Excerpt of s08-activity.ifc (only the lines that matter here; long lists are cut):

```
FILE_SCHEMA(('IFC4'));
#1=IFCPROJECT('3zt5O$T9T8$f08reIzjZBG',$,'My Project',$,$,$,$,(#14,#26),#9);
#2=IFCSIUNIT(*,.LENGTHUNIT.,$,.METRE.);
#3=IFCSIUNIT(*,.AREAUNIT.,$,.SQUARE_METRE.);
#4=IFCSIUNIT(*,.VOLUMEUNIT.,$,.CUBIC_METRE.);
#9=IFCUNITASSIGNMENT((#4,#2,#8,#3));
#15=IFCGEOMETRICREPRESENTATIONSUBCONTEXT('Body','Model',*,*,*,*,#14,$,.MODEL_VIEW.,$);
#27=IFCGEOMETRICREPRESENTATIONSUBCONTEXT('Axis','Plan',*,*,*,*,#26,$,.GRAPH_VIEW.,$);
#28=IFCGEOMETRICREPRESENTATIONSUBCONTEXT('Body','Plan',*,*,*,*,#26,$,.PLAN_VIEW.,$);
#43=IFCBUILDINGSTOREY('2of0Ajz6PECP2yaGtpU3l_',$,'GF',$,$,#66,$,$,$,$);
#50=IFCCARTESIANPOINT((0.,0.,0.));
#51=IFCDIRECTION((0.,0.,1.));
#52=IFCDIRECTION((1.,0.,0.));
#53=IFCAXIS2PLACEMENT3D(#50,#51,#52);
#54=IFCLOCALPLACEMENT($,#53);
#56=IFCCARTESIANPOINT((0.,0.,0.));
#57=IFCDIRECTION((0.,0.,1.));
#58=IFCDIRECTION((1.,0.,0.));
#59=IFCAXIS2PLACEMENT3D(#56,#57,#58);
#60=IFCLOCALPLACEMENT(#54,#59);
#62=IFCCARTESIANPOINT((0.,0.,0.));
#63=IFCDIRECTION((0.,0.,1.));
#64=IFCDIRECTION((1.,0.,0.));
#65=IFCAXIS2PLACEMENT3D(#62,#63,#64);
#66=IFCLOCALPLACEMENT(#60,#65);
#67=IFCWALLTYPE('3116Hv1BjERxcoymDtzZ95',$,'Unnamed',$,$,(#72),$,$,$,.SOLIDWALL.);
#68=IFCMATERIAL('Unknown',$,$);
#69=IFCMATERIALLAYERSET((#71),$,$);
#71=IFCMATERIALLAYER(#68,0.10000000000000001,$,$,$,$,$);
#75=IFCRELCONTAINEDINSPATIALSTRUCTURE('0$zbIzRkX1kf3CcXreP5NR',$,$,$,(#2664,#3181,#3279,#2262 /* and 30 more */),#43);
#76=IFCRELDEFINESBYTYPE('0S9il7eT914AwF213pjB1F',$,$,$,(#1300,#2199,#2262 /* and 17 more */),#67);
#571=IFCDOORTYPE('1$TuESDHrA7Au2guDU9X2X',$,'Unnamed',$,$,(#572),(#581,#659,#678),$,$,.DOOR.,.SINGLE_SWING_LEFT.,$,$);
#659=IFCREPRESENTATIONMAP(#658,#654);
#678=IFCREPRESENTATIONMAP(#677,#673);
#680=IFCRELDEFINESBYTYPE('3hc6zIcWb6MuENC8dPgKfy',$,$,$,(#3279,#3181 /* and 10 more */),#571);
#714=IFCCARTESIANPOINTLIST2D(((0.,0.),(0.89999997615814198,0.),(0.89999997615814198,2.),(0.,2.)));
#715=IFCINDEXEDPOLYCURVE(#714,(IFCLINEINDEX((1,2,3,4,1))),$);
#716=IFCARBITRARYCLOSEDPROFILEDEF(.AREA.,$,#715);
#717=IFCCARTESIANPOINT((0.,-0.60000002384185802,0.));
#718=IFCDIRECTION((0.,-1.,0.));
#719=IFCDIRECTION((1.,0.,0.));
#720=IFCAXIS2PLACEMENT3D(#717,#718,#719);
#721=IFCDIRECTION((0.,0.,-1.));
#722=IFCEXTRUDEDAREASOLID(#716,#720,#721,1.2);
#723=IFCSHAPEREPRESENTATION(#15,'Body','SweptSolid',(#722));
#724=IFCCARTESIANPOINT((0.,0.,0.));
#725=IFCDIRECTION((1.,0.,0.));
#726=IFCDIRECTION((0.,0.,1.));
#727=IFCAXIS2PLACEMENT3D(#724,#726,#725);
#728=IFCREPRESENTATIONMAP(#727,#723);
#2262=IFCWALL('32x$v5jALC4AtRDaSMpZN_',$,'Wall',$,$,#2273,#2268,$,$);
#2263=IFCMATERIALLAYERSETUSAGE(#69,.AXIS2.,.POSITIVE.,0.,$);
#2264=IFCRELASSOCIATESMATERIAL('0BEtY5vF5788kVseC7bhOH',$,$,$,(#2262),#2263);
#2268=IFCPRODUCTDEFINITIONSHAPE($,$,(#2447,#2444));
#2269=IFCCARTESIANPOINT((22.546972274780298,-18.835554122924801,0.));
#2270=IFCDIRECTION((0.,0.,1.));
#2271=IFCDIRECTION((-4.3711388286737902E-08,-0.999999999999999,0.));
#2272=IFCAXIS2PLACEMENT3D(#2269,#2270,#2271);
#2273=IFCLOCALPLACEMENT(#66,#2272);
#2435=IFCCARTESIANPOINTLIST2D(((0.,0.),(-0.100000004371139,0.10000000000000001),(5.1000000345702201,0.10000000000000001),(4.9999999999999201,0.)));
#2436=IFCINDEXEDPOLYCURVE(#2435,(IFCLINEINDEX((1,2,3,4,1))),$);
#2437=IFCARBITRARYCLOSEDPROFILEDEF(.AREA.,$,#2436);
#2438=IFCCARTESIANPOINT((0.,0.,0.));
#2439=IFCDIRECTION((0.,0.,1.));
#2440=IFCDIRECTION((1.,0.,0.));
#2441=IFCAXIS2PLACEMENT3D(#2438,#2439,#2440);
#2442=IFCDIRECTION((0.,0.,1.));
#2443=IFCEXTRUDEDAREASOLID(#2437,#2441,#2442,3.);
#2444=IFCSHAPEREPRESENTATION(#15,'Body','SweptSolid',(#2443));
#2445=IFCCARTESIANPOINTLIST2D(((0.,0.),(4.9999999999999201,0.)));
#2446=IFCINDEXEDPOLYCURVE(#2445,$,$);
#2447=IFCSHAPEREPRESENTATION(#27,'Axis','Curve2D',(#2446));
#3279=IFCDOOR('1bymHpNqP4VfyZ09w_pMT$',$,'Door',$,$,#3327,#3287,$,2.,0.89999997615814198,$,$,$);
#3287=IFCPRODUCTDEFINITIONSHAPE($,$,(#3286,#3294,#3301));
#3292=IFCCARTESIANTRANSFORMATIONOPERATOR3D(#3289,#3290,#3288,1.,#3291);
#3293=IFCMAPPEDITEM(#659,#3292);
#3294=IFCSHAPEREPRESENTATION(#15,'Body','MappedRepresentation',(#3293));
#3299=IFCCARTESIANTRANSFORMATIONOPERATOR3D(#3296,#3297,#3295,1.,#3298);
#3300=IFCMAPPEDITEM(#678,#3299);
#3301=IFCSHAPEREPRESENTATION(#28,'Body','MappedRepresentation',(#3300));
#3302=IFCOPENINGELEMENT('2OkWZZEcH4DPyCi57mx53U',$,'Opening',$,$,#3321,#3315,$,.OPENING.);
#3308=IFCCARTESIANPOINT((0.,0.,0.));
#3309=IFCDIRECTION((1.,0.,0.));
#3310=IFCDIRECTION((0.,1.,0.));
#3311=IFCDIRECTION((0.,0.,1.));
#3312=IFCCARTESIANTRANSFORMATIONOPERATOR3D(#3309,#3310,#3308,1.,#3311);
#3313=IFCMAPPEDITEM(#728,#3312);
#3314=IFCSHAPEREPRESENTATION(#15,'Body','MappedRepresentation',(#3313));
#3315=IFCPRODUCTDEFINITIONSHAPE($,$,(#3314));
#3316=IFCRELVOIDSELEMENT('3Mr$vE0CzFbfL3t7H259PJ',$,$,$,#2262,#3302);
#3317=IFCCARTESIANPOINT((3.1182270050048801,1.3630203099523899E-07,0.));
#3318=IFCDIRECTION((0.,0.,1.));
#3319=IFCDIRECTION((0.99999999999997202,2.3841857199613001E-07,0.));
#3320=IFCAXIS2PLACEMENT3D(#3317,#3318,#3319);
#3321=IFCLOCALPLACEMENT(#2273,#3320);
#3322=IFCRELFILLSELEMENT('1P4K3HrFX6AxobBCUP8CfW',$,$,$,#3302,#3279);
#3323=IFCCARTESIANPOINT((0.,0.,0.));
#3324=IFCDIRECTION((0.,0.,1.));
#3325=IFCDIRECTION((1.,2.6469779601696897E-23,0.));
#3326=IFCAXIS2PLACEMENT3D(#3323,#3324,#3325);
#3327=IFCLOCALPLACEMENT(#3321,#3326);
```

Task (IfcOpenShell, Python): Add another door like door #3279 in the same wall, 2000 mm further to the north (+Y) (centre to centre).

```python
import ifcopenshell
import ifcopenshell.api.feature
import ifcopenshell.api.geometry
import ifcopenshell.api.root
import ifcopenshell.geom
import ifcopenshell.util.element
import ifcopenshell.util.placement
import ifcopenshell.util.shape
import ifcopenshell.util.unit

model = ifcopenshell.open("s08-activity.ifc")
unit_scale = ifcopenshell.util.unit.calculate_unit_scale(model)
settings = ifcopenshell.geom.settings()


def volume(element):
    """Net volume in cubic metres, openings subtracted."""
    shape = ifcopenshell.geom.create_shape(settings, element)
    return ifcopenshell.util.shape.get_volume(shape.geometry)


door = model.by_id(3279)
opening = door.FillsVoids[0].RelatingOpeningElement
wall = opening.VoidsElements[0].RelatingBuildingElement
before = volume(wall)
shift = ifcopenshell.util.placement.get_local_placement(wall.ObjectPlacement)[:3, 0] * -2 / unit_scale

# copy_class copies the void relationship, type, container and properties, but no geometry.
new_opening = ifcopenshell.api.root.copy_class(model, product=opening)
new_opening.Representation = ifcopenshell.util.element.copy_deep(
    model, opening.Representation, exclude=["IfcGeometricRepresentationContext", "IfcRepresentationMap"]
)
new_door = ifcopenshell.api.root.copy_class(model, product=door)
new_door.Representation = ifcopenshell.util.element.copy_deep(
    model, door.Representation, exclude=["IfcGeometricRepresentationContext", "IfcRepresentationMap"]
)
ifcopenshell.api.feature.add_filling(model, opening=new_opening, element=new_door)

for old, new in ((opening, new_opening), (door, new_door)):
    matrix = ifcopenshell.util.placement.get_local_placement(old.ObjectPlacement)
    matrix[:3, 3] += shift
    ifcopenshell.api.geometry.edit_object_placement(model, product=new, matrix=matrix, is_si=False)

after = volume(wall)

print(f"wall volume {before:.3f} -> {after:.3f} m3")

model.write("s08-activity_rev.ifc")
```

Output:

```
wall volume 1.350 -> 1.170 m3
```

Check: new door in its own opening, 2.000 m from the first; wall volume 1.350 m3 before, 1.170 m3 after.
